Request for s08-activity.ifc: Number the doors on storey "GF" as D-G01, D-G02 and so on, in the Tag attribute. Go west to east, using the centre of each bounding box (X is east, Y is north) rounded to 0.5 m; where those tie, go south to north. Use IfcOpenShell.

First a look at what the model holds.

```python
import ifcopenshell
import ifcopenshell.util.element
import ifcopenshell.util.placement

model = ifcopenshell.open("s08-activity.ifc")
print(model.schema)
storey = next(s for s in model.by_type("IfcBuildingStorey") if s.Name == "GF")
doors = [e for e in ifcopenshell.util.element.get_decomposition(storey) if e.is_a("IfcDoor")]
for e in sorted(doors, key=lambda e: e.id()):
    origin = ifcopenshell.util.placement.get_local_placement(e.ObjectPlacement)[:3, 3]
    print(e.id(), e.Tag, e.Name, origin.round(2) + 0.0, sep=" | ")
```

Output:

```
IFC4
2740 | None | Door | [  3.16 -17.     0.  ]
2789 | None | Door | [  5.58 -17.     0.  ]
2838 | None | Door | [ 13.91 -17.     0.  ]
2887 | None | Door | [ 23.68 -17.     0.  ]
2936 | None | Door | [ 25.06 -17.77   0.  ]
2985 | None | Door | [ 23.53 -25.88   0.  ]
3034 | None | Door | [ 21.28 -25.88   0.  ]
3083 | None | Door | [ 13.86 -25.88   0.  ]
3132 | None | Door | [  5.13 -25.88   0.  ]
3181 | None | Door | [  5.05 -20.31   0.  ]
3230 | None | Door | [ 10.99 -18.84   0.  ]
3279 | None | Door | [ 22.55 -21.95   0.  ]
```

```python
import ifcopenshell
import ifcopenshell.geom
import ifcopenshell.util.element
import ifcopenshell.util.shape

model = ifcopenshell.open("s08-activity.ifc")
settings = ifcopenshell.geom.settings()
settings.set("use-world-coords", True)


def centre(element):
    shape = ifcopenshell.geom.create_shape(settings, element)
    return ifcopenshell.util.shape.get_bbox_centroid(shape.geometry)


storey = next(s for s in model.by_type("IfcBuildingStorey") if s.Name == "GF")
doors = [e for e in ifcopenshell.util.element.get_decomposition(storey) if e.is_a("IfcDoor")]

# Insertion points can sit at a corner or the storey origin, so sort by the geometry (in metres).
centres = {e: centre(e) for e in doors}
doors.sort(key=lambda e: (round(centres[e][0] / 0.5), centres[e][1]))

for i, e in enumerate(doors, start=1):
    number = f"D-G{i:02d}"
    e.Tag = number
    print(e.id(), number)

model.write("s08-activity_rev.ifc")
```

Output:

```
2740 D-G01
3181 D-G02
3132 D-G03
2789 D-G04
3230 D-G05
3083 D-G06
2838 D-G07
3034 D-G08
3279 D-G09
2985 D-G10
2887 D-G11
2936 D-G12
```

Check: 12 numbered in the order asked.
